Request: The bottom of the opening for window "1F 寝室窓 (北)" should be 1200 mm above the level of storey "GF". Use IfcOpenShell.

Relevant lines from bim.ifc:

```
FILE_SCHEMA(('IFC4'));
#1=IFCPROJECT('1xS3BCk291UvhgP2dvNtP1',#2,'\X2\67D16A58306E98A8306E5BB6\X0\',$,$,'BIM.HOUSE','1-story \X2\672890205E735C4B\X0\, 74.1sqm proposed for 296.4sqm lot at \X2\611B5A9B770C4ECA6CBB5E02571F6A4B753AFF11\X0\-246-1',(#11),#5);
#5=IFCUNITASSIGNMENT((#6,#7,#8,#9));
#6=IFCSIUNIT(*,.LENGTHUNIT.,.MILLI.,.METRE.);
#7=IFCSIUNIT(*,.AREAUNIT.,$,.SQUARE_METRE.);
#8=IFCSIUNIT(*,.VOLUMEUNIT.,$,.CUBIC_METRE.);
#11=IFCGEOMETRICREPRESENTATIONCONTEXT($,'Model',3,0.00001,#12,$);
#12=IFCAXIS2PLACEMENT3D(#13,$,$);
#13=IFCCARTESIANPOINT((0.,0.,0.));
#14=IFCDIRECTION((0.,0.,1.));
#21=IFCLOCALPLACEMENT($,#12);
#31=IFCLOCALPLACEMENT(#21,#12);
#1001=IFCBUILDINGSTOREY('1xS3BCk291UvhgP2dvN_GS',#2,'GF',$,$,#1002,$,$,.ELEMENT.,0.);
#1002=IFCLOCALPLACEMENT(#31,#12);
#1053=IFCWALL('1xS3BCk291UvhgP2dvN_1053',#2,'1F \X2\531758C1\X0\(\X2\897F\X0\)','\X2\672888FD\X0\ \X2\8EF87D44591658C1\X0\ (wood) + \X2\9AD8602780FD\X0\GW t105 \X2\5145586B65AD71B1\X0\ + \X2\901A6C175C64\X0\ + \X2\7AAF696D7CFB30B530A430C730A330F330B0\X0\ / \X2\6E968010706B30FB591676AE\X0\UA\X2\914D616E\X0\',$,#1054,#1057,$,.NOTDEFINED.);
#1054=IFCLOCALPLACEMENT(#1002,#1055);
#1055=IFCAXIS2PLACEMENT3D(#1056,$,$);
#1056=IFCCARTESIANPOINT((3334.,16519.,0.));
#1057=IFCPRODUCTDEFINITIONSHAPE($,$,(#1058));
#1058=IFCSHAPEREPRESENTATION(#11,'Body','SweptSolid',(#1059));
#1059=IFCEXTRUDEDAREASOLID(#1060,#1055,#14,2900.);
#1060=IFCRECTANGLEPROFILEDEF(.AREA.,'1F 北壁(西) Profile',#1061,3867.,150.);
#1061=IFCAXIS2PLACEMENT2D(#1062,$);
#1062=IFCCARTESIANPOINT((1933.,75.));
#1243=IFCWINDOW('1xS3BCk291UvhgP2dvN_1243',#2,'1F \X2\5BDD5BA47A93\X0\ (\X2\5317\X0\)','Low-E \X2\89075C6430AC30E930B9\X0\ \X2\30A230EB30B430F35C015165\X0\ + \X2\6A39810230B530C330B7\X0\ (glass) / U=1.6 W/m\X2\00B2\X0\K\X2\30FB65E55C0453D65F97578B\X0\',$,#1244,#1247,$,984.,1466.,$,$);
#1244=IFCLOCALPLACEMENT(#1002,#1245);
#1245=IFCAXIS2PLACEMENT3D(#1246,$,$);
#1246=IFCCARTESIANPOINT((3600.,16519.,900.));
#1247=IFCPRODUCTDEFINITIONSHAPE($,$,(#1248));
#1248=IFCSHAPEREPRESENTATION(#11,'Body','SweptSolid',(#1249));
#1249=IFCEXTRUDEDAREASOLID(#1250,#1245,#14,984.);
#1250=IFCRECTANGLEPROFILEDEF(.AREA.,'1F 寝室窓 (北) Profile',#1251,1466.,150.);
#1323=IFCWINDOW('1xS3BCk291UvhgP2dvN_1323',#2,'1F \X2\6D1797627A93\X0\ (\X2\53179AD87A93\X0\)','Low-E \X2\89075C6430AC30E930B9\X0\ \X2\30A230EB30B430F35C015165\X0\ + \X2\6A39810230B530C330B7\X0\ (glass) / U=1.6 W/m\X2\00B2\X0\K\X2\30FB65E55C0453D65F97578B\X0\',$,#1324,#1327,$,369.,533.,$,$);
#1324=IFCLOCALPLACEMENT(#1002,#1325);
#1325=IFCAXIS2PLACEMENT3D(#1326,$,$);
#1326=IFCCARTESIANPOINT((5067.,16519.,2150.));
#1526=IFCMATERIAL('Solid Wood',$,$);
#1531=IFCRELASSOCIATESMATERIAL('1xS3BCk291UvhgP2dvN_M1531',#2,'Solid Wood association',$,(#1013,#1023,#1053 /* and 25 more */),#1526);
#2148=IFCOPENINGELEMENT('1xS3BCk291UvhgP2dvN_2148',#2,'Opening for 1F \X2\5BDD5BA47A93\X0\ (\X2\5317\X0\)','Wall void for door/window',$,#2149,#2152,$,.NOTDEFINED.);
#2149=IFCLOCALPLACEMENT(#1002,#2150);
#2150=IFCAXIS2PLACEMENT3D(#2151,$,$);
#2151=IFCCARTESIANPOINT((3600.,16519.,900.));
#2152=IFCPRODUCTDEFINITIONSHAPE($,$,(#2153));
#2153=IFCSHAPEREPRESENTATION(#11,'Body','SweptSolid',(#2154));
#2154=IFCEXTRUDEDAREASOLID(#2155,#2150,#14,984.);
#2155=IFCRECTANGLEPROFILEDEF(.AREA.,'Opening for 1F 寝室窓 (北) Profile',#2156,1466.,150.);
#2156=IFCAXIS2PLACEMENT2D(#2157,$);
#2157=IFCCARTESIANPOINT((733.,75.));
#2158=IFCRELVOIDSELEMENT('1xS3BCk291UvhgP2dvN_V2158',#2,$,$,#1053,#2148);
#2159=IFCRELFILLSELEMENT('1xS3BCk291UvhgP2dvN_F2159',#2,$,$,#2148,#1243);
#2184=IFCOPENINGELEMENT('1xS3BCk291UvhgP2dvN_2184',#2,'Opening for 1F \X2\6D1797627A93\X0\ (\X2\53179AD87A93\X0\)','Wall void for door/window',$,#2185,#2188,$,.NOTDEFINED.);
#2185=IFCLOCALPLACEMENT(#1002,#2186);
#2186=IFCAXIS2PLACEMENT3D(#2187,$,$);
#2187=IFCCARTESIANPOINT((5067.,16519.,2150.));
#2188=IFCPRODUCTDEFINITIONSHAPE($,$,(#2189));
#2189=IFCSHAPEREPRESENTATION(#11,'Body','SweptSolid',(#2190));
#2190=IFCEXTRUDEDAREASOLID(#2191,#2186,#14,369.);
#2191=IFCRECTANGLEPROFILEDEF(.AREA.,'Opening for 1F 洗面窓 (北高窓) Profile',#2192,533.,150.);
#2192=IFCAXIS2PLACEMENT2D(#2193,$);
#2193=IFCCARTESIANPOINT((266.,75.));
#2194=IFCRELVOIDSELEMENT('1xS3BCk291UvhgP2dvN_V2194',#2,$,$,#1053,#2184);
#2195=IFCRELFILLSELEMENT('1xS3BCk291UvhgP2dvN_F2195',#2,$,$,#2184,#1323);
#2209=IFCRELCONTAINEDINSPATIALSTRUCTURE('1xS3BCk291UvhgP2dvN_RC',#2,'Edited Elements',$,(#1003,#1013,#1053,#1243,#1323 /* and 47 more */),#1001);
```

```python
import numpy as np
import ifcopenshell
import ifcopenshell.api.geometry
import ifcopenshell.geom
import ifcopenshell.util.element
import ifcopenshell.util.placement
import ifcopenshell.util.shape
import ifcopenshell.util.unit

model = ifcopenshell.open("bim.ifc")
unit_scale = ifcopenshell.util.unit.calculate_unit_scale(model)

window = model.by_guid("1xS3BCk291UvhgP2dvN_1243")
opening = window.FillsVoids[0].RelatingOpeningElement
storey = ifcopenshell.util.element.get_container(window, ifc_class="IfcBuildingStorey")
level = ifcopenshell.util.placement.get_local_placement(storey.ObjectPlacement)[2, 3]

# The opening's origin need not be at the sill, so measure its lowest point.
shape = ifcopenshell.geom.create_shape(ifcopenshell.geom.settings(), opening)
bottom = ifcopenshell.util.shape.get_shape_bottom_elevation(shape, shape.geometry) / unit_scale
dz = level + 1200.0 - bottom

shift = np.array([0.0, 0.0, dz])
# The window is not placed relative to its opening, so move both.
for product in (opening, window):
    matrix = ifcopenshell.util.placement.get_local_placement(product.ObjectPlacement)
    matrix[:3, 3] += shift
    ifcopenshell.api.geometry.edit_object_placement(model, product=product, matrix=matrix, is_si=False)

print(f"moved by {dz * unit_scale:+.3f} m")

model.write("bim_rev.ifc")
```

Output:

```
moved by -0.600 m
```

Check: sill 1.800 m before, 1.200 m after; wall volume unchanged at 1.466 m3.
